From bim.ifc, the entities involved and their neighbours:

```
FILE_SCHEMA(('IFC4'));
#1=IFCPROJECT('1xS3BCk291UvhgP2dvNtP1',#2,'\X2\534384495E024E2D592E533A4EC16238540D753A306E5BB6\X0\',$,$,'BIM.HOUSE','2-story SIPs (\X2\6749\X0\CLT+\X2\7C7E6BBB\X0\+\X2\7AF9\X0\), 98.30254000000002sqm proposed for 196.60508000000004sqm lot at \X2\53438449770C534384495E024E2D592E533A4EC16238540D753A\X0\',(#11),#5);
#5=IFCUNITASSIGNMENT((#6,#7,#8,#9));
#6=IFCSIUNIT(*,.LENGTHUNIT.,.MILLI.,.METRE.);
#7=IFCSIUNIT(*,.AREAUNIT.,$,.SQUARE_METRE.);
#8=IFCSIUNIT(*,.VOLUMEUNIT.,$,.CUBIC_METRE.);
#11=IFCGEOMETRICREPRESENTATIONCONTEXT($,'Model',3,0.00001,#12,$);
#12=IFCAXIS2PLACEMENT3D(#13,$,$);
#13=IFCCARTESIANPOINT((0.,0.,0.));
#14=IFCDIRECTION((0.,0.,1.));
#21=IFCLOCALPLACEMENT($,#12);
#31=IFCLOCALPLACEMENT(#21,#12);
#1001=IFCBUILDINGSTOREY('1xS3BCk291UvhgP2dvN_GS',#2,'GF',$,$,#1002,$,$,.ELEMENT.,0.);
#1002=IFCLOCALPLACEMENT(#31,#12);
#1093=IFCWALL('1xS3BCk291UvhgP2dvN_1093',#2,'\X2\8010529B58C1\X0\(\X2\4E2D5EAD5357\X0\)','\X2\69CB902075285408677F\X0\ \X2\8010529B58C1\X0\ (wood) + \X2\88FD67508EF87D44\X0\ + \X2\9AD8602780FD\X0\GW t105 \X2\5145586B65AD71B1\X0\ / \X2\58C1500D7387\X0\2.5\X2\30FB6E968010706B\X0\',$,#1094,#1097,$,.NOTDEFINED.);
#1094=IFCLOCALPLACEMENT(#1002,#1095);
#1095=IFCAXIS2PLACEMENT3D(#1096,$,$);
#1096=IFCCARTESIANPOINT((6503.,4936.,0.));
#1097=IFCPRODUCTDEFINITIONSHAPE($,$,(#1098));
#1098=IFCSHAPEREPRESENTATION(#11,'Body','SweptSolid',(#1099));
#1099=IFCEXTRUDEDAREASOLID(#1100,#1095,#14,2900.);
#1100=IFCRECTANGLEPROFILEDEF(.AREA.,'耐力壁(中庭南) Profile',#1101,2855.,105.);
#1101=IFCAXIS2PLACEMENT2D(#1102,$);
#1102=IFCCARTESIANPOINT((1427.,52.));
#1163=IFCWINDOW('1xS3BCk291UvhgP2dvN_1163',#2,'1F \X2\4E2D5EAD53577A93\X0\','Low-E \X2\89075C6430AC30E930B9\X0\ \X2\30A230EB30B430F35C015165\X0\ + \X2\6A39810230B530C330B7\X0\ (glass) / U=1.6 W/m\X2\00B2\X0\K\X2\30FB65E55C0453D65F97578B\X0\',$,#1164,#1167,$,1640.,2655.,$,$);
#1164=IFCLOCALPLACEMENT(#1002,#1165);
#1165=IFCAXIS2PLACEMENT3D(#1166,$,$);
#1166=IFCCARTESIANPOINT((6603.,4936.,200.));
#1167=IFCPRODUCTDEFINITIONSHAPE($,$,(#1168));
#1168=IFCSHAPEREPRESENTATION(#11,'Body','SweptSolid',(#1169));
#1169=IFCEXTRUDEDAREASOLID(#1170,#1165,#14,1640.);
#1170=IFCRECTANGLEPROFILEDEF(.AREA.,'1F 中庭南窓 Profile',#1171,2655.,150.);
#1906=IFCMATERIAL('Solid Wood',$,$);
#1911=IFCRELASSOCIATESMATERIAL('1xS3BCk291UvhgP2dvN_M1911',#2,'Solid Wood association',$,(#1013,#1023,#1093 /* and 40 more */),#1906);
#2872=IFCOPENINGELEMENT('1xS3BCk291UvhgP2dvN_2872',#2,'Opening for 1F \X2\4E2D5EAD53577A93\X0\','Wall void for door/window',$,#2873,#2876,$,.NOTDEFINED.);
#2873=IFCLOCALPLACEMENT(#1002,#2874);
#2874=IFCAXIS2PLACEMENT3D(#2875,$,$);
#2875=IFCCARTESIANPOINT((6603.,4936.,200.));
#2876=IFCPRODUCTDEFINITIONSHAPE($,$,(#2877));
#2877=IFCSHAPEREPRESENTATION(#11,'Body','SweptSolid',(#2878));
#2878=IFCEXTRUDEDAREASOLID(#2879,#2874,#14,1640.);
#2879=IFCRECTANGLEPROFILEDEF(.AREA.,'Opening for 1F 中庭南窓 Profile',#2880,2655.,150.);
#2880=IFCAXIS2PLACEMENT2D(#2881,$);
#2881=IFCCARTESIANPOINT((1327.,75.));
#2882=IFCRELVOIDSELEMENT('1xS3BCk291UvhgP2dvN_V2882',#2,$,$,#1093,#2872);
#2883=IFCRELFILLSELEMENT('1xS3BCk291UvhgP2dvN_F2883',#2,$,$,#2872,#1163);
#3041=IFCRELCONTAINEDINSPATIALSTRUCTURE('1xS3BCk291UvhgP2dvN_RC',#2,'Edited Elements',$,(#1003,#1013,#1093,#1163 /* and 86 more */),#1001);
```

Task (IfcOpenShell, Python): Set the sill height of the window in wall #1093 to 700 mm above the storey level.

```python
import numpy as np
import ifcopenshell
import ifcopenshell.api.geometry
import ifcopenshell.geom
import ifcopenshell.util.element
import ifcopenshell.util.placement
import ifcopenshell.util.shape
import ifcopenshell.util.unit

model = ifcopenshell.open("bim.ifc")
unit_scale = ifcopenshell.util.unit.calculate_unit_scale(model)

window = model.by_guid("1xS3BCk291UvhgP2dvN_1163")
opening = window.FillsVoids[0].RelatingOpeningElement
storey = ifcopenshell.util.element.get_container(window, ifc_class="IfcBuildingStorey")
level = ifcopenshell.util.placement.get_local_placement(storey.ObjectPlacement)[2, 3]

# The opening's origin need not be at the sill, so measure its lowest point.
shape = ifcopenshell.geom.create_shape(ifcopenshell.geom.settings(), opening)
bottom = ifcopenshell.util.shape.get_shape_bottom_elevation(shape, shape.geometry) / unit_scale
dz = level + 700.0 - bottom

shift = np.array([0.0, 0.0, dz])
# The window is not placed relative to its opening, so move both.
for product in (opening, window):
    matrix = ifcopenshell.util.placement.get_local_placement(product.ObjectPlacement)
    matrix[:3, 3] += shift
    ifcopenshell.api.geometry.edit_object_placement(model, product=product, matrix=matrix, is_si=False)

print(f"moved by {dz * unit_scale:+.3f} m")

model.write("bim_rev.ifc")
```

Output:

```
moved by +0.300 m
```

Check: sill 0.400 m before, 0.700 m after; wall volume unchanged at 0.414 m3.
